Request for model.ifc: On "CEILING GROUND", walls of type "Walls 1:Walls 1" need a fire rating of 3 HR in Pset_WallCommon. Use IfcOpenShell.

First a look at what the model holds.

```python
import ifcopenshell
import ifcopenshell.util.element

model = ifcopenshell.open("model.ifc")
print(model.schema)
storey = next(s for s in model.by_type("IfcBuildingStorey") if s.Name == "CEILING GROUND")
walls = [e for e in ifcopenshell.util.element.get_decomposition(storey) if e.is_a("IfcWall")]
seen = {}
for e in walls:
    element_type = ifcopenshell.util.element.get_type(e)
    key = (element_type.Name if element_type != e and element_type else None, ifcopenshell.util.element.get_pset(e, "Pset_WallCommon", "FireRating"))
    seen[key] = seen.get(key, 0) + 1
for (name, value), count in sorted(seen.items(), key=str):
    print(count, "x", name, "|", value)
```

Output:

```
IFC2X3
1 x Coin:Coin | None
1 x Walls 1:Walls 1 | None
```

```python
import ifcopenshell
import ifcopenshell.api.pset
import ifcopenshell.util.element

model = ifcopenshell.open("model.ifc")

storey = next(s for s in model.by_type("IfcBuildingStorey") if s.Name == "CEILING GROUND")
walls = [e for e in ifcopenshell.util.element.get_decomposition(storey) if e.is_a("IfcWall")]

count = 0
for e in walls:
    element_type = ifcopenshell.util.element.get_type(e)
    if element_type in (None, e) or element_type.Name != "Walls 1:Walls 1":
        continue
    # add_pset returns the element's existing set when there is one.
    pset = ifcopenshell.api.pset.add_pset(model, product=e, name="Pset_WallCommon")
    ifcopenshell.api.pset.edit_pset(model, pset=pset, properties={"FireRating": "3 HR"})
    count += 1

print(count, "walls updated")

model.write("model_updated.ifc")
```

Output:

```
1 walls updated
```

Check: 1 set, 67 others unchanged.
